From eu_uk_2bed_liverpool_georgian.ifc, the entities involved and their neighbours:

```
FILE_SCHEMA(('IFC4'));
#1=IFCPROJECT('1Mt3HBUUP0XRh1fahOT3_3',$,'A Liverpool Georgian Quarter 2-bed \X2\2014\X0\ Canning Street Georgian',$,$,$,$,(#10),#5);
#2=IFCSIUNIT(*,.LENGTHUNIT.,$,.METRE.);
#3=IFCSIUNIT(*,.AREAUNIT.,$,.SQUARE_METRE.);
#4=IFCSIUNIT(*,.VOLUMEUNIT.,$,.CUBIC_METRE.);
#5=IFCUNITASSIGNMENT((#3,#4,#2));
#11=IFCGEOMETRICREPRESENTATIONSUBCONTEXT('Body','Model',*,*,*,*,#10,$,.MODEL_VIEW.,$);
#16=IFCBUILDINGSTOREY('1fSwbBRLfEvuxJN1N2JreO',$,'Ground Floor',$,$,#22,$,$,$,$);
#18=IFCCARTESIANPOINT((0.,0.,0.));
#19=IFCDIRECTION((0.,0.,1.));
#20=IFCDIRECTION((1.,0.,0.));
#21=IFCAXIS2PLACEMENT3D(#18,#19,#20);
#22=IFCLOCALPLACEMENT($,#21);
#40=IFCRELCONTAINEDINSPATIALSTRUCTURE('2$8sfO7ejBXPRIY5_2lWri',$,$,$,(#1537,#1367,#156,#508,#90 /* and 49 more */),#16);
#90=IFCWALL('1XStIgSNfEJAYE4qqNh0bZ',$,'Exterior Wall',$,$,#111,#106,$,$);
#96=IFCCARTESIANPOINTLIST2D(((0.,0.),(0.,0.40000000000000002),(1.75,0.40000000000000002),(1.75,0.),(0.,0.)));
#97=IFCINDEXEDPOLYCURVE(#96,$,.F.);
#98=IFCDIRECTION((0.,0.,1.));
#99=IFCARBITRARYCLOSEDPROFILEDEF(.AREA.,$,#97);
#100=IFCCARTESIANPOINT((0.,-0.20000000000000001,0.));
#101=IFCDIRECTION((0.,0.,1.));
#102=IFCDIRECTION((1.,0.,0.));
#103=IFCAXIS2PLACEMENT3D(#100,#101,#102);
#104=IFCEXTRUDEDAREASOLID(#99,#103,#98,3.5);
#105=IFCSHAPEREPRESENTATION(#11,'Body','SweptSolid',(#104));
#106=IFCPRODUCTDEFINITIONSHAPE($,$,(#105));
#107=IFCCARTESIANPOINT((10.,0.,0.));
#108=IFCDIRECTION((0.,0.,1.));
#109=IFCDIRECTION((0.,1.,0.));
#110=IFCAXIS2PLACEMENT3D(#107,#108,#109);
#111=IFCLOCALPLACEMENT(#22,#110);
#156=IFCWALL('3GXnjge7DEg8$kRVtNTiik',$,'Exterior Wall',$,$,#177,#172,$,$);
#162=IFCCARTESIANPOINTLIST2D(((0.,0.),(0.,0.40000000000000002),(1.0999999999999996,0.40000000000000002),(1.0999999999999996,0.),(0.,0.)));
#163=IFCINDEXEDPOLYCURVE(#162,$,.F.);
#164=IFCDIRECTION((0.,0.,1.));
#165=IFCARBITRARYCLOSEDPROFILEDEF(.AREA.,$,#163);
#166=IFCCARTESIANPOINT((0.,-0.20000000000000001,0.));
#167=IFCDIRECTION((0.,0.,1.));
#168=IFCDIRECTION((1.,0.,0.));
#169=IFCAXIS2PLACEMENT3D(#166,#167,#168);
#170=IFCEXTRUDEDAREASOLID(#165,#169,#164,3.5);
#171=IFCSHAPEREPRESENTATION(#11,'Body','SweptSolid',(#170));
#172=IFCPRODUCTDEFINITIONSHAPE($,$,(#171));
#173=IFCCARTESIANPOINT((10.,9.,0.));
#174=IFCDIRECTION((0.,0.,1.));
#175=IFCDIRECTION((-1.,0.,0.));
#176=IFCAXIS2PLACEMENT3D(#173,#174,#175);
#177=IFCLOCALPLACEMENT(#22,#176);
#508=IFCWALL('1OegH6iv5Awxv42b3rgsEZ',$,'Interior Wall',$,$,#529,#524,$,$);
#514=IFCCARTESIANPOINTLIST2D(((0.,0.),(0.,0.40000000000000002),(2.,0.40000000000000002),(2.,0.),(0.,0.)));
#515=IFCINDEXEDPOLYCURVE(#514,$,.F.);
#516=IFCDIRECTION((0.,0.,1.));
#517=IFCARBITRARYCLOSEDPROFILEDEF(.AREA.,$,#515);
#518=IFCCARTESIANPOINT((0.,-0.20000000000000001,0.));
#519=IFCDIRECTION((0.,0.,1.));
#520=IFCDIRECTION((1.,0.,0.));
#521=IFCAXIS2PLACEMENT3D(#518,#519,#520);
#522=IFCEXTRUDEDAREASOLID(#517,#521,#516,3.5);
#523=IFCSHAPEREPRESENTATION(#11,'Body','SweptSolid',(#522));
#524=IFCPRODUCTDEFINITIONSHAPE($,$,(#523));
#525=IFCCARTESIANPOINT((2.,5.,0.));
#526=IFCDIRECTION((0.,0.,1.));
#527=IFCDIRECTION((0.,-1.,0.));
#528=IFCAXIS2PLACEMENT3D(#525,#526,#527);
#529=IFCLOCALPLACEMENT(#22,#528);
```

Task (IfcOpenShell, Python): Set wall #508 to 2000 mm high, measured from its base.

```python
import ifcopenshell
import ifcopenshell.geom
import ifcopenshell.util.representation
import ifcopenshell.util.shape
import ifcopenshell.util.unit

model = ifcopenshell.open("eu_uk_2bed_liverpool_georgian.ifc")
unit_scale = ifcopenshell.util.unit.calculate_unit_scale(model)
settings = ifcopenshell.geom.settings()


def volume(element):
    """Net volume in cubic metres, openings subtracted."""
    shape = ifcopenshell.geom.create_shape(settings, element)
    return ifcopenshell.util.shape.get_volume(shape.geometry)


wall = model.by_guid("1OegH6iv5Awxv42b3rgsEZ")
before = volume(wall)

body = ifcopenshell.util.representation.get_representation(wall, "Model", "Body")
solid = body.Items[0]
old_height = solid.Depth
solid.Depth = 2 / unit_scale
after = volume(wall)

print(f"height {old_height:g} -> {solid.Depth:g}, volume {before:.3f} -> {after:.3f} m3")

model.write("eu_uk_2bed_liverpool_georgian_updated.ifc")
```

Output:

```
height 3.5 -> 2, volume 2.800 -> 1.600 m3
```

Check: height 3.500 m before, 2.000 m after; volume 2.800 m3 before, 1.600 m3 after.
